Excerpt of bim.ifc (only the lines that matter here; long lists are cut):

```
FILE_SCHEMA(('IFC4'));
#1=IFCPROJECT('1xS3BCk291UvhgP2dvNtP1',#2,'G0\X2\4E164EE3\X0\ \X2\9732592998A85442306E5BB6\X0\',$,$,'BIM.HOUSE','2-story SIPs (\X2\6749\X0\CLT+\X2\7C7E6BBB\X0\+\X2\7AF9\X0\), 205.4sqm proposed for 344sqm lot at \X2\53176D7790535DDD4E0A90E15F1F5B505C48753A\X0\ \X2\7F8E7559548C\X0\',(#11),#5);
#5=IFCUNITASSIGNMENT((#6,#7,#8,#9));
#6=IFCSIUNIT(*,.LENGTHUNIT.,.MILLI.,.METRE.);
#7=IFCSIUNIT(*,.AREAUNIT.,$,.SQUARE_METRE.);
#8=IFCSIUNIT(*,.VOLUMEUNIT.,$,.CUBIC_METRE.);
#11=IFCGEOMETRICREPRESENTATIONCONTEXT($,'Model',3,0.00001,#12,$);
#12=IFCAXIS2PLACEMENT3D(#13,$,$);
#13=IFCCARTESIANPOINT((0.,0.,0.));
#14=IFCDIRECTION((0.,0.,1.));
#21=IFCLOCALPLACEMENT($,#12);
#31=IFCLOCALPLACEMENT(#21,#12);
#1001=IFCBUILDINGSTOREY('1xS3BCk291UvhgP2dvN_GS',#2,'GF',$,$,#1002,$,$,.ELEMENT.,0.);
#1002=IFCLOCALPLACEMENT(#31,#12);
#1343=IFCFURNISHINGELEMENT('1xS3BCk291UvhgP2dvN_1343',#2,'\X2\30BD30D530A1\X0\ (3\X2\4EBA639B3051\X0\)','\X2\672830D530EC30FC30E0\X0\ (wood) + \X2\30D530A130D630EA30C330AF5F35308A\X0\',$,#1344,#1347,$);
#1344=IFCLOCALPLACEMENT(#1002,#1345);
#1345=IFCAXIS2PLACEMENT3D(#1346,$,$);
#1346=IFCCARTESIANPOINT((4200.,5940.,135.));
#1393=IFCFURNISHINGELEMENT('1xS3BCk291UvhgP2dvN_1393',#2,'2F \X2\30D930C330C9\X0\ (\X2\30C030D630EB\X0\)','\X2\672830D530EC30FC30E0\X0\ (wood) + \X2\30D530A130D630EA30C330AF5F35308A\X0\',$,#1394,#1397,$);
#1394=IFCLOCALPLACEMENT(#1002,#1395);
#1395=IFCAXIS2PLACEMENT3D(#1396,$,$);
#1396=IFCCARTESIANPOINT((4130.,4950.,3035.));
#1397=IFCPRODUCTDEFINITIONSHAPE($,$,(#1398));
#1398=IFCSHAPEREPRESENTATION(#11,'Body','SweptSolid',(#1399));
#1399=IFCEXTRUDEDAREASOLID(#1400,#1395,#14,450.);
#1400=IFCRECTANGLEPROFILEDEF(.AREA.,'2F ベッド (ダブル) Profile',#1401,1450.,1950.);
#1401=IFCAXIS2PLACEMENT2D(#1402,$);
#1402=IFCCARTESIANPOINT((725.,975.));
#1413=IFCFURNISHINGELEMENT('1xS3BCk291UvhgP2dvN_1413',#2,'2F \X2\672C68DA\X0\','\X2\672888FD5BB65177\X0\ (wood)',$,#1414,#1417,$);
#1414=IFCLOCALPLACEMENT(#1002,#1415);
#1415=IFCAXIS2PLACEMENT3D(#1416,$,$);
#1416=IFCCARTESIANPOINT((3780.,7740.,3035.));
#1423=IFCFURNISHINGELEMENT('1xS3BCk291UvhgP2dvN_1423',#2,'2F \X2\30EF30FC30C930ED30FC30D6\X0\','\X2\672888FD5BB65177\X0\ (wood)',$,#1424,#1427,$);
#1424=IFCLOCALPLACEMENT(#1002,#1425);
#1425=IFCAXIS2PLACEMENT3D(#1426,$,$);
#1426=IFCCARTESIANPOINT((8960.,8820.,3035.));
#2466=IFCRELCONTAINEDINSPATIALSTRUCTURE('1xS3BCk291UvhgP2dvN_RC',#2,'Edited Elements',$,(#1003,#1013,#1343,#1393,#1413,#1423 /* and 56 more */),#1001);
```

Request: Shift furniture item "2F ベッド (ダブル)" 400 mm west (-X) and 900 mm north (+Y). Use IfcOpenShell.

```python
import ifcopenshell
import ifcopenshell.api.geometry
import ifcopenshell.util.placement

model = ifcopenshell.open("bim.ifc")

item = model.by_id(1393)
matrix = ifcopenshell.util.placement.get_local_placement(item.ObjectPlacement)
matrix[0, 3] -= 400.0
matrix[1, 3] += 900.0
ifcopenshell.api.geometry.edit_object_placement(model, product=item, matrix=matrix, is_si=False)

print(ifcopenshell.util.placement.get_local_placement(item.ObjectPlacement).round(3) + 0.0)

model.write("bim-out.ifc")
```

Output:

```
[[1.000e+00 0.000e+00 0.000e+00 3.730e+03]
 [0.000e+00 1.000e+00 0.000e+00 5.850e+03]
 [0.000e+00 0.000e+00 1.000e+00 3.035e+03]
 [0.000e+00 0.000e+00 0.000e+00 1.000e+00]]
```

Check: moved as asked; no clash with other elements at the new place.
